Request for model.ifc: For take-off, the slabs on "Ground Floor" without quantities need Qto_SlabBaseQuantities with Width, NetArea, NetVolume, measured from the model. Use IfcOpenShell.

First a look at what the model holds.

```python
import ifcopenshell
import ifcopenshell.util.element
import ifcopenshell.util.unit

model = ifcopenshell.open("model.ifc")
print(model.schema)
for unit_type in ("LENGTHUNIT", "AREAUNIT", "VOLUMEUNIT"):
    print(unit_type, ifcopenshell.util.unit.calculate_unit_scale(model, unit_type))
storey = next(s for s in model.by_type("IfcBuildingStorey") if s.Name == "Ground Floor")
slabs = [e for e in ifcopenshell.util.element.get_decomposition(storey) if e.is_a("IfcSlab")]
for e in sorted(slabs, key=lambda e: e.id()):
    print(e.id(), e.is_a(), e.Name, list(ifcopenshell.util.element.get_psets(e, qtos_only=True)), sep=" | ")
```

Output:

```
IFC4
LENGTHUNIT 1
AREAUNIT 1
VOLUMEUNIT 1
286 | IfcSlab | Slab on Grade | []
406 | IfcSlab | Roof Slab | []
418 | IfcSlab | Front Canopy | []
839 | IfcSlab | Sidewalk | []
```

```python
import ifcopenshell
import ifcopenshell.api.pset
import ifcopenshell.geom
import ifcopenshell.util.element
import ifcopenshell.util.shape
import ifcopenshell.util.unit

model = ifcopenshell.open("model.ifc")
unit_scale = ifcopenshell.util.unit.calculate_unit_scale(model)
area_scale = ifcopenshell.util.unit.calculate_unit_scale(model, "AREAUNIT")
volume_scale = ifcopenshell.util.unit.calculate_unit_scale(model, "VOLUMEUNIT")
settings = ifcopenshell.geom.settings()

storey = next(s for s in model.by_type("IfcBuildingStorey") if s.Name == "Ground Floor")
slabs = [e for e in ifcopenshell.util.element.get_decomposition(storey) if e.is_a("IfcSlab")]

for e in sorted(slabs, key=lambda e: e.id()):
    if ifcopenshell.util.element.get_psets(e, qtos_only=True, should_inherit=False):
        continue
    # Geometry comes back in metres, in the element's own axes.
    shape = ifcopenshell.geom.create_shape(settings, e)
    values = {
        "Width": ifcopenshell.util.shape.get_z(shape.geometry) / unit_scale,
        "NetArea": ifcopenshell.util.shape.get_footprint_area(shape.geometry) / area_scale,
        "NetVolume": ifcopenshell.util.shape.get_volume(shape.geometry) / volume_scale,
    }
    qto = ifcopenshell.api.pset.add_qto(model, product=e, name="Qto_SlabBaseQuantities")
    ifcopenshell.api.pset.edit_qto(model, qto=qto, properties=values)
    print(e.id(), {k: round(v, 3) for k, v in values.items()})

model.write("model-out.ifc")
```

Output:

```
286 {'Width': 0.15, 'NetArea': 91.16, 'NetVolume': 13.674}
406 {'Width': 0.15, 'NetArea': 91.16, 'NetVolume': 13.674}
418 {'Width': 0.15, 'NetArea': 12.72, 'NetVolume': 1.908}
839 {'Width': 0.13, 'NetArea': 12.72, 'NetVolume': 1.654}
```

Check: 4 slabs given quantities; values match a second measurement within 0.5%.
